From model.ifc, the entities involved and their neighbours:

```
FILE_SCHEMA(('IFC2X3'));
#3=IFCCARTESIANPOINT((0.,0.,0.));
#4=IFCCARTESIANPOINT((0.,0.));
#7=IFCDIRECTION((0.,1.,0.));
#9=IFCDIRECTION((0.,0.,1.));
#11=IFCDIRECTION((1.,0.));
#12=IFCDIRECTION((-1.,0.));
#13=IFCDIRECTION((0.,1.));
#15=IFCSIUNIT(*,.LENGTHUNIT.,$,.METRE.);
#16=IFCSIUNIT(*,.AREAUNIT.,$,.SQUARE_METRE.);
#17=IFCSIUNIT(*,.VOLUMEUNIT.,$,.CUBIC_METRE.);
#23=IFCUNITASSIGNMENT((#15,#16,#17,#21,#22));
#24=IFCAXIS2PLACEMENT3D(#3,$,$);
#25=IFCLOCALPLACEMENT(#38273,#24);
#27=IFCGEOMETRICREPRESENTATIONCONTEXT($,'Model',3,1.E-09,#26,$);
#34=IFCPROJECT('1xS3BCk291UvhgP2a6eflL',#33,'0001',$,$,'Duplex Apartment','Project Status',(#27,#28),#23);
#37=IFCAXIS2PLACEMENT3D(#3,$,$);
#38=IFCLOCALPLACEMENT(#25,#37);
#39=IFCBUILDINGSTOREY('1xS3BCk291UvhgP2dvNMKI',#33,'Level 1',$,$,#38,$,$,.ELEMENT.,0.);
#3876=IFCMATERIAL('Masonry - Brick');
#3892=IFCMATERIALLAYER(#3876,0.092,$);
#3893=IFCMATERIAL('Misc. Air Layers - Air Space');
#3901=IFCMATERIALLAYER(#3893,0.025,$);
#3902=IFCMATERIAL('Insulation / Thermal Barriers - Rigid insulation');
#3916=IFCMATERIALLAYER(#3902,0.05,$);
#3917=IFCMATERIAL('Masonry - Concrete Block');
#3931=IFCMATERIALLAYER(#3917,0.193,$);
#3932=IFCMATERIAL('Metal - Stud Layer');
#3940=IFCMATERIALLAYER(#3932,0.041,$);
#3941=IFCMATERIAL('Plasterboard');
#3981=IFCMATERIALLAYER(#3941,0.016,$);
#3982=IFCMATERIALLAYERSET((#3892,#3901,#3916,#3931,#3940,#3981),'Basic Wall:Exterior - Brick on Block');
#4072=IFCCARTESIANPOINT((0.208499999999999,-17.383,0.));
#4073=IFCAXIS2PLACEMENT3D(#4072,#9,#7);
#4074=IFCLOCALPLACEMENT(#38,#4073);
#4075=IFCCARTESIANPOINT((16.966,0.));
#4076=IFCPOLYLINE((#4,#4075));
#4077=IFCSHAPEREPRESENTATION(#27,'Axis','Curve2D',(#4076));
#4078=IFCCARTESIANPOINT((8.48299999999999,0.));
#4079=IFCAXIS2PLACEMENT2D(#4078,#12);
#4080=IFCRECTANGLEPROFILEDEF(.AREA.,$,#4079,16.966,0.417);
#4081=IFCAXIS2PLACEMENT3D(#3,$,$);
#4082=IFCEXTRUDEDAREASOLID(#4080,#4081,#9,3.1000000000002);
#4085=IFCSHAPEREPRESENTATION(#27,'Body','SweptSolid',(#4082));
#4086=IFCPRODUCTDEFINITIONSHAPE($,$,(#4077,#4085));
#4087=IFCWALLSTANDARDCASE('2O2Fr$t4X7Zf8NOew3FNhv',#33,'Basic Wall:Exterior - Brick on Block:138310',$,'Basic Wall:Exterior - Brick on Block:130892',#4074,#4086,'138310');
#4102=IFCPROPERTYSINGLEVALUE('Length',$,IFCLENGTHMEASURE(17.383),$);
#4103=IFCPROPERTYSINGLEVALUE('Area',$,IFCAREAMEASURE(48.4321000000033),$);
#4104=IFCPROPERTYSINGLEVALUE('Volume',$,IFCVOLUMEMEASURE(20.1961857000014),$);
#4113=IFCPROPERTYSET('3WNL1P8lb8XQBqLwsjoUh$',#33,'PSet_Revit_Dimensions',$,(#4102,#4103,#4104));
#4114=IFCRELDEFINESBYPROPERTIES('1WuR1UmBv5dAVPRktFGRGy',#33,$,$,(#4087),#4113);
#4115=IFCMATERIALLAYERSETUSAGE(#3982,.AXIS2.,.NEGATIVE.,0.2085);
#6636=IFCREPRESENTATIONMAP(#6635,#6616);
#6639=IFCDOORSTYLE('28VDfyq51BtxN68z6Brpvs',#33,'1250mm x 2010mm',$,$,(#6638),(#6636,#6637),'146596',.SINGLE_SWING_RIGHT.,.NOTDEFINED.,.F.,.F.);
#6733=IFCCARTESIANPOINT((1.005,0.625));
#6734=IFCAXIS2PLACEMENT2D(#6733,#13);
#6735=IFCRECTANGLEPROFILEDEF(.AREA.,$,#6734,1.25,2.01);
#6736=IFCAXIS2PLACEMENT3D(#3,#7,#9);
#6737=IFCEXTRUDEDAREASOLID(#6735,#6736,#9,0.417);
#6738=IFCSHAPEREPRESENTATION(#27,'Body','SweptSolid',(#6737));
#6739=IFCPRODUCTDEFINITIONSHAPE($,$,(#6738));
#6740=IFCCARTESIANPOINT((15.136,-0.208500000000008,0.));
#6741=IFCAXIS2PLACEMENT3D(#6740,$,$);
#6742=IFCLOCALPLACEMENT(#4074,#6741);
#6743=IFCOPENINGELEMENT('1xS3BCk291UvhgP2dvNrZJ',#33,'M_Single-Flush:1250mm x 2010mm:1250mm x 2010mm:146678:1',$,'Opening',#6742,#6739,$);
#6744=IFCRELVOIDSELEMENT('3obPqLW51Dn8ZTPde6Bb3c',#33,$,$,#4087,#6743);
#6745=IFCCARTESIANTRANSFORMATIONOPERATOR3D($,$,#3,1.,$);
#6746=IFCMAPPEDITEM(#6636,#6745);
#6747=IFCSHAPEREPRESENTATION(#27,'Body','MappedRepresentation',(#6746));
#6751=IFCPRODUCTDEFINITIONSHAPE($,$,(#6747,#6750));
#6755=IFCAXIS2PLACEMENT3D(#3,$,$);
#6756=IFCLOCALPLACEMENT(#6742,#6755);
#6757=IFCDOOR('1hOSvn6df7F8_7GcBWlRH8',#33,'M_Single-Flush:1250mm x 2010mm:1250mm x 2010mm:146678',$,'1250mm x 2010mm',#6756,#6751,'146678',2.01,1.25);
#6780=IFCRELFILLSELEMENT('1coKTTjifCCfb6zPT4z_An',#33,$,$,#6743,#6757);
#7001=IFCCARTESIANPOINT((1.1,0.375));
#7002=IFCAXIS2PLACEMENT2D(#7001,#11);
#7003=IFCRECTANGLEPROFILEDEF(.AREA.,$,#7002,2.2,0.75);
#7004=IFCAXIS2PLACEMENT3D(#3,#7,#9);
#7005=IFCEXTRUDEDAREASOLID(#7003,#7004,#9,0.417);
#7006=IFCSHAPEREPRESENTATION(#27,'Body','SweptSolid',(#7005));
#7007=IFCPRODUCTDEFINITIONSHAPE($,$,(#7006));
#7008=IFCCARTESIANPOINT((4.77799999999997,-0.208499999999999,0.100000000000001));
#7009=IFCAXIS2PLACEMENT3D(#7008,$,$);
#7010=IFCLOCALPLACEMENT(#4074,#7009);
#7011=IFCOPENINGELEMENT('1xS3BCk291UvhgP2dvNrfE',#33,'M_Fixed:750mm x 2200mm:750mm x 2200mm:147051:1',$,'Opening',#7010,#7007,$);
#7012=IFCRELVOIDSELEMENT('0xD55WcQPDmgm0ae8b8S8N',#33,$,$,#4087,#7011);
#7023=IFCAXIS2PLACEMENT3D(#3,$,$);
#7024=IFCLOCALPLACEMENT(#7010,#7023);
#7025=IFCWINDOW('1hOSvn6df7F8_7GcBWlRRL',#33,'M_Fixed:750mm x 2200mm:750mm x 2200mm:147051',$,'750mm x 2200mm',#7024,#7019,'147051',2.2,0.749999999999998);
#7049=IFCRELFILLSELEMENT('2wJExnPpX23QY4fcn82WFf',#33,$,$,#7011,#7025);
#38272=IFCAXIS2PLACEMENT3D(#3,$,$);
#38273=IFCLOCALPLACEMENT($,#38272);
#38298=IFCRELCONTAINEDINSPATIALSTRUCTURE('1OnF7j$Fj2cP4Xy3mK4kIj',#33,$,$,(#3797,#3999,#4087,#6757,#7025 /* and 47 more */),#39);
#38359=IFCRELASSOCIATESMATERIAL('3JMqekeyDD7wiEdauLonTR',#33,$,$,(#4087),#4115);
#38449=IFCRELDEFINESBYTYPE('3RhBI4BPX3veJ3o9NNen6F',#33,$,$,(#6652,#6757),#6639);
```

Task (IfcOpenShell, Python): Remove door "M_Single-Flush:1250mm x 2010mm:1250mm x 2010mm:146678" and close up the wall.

```python
import ifcopenshell
import ifcopenshell.api.feature
import ifcopenshell.api.pset
import ifcopenshell.api.root
import ifcopenshell.geom
import ifcopenshell.util.element
import ifcopenshell.util.shape
import ifcopenshell.util.unit

model = ifcopenshell.open("model.ifc")
area_scale = ifcopenshell.util.unit.calculate_unit_scale(model, "AREAUNIT")
volume_scale = ifcopenshell.util.unit.calculate_unit_scale(model, "VOLUMEUNIT")
settings = ifcopenshell.geom.settings()


def volume(element):
    """Net volume in cubic metres, openings subtracted."""
    shape = ifcopenshell.geom.create_shape(settings, element)
    return ifcopenshell.util.shape.get_volume(shape.geometry)


door = model.by_guid("1hOSvn6df7F8_7GcBWlRH8")
opening = door.FillsVoids[0].RelatingOpeningElement
wall = opening.VoidsElements[0].RelatingBuildingElement
before = volume(wall)

ifcopenshell.api.root.remove_product(model, product=door)
ifcopenshell.api.feature.remove_feature(model, feature=opening)

after = volume(wall)
thickness = 0.417  # wall thickness in metres

# Update the wall's stored quantities.
pset = model.by_id(ifcopenshell.util.element.get_pset(wall, "PSet_Revit_Dimensions", should_inherit=False)["id"])
ifcopenshell.api.pset.edit_pset(model, pset=pset, properties={
    "Area": model.create_entity("IfcAreaMeasure", after / thickness / area_scale),
    "Volume": model.create_entity("IfcVolumeMeasure", after / volume_scale),
})

print(f"wall volume {before:.3f} -> {after:.3f} m3")

model.write("model_edited.ifc")
```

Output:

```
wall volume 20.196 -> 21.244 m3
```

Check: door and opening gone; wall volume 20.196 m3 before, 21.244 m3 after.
